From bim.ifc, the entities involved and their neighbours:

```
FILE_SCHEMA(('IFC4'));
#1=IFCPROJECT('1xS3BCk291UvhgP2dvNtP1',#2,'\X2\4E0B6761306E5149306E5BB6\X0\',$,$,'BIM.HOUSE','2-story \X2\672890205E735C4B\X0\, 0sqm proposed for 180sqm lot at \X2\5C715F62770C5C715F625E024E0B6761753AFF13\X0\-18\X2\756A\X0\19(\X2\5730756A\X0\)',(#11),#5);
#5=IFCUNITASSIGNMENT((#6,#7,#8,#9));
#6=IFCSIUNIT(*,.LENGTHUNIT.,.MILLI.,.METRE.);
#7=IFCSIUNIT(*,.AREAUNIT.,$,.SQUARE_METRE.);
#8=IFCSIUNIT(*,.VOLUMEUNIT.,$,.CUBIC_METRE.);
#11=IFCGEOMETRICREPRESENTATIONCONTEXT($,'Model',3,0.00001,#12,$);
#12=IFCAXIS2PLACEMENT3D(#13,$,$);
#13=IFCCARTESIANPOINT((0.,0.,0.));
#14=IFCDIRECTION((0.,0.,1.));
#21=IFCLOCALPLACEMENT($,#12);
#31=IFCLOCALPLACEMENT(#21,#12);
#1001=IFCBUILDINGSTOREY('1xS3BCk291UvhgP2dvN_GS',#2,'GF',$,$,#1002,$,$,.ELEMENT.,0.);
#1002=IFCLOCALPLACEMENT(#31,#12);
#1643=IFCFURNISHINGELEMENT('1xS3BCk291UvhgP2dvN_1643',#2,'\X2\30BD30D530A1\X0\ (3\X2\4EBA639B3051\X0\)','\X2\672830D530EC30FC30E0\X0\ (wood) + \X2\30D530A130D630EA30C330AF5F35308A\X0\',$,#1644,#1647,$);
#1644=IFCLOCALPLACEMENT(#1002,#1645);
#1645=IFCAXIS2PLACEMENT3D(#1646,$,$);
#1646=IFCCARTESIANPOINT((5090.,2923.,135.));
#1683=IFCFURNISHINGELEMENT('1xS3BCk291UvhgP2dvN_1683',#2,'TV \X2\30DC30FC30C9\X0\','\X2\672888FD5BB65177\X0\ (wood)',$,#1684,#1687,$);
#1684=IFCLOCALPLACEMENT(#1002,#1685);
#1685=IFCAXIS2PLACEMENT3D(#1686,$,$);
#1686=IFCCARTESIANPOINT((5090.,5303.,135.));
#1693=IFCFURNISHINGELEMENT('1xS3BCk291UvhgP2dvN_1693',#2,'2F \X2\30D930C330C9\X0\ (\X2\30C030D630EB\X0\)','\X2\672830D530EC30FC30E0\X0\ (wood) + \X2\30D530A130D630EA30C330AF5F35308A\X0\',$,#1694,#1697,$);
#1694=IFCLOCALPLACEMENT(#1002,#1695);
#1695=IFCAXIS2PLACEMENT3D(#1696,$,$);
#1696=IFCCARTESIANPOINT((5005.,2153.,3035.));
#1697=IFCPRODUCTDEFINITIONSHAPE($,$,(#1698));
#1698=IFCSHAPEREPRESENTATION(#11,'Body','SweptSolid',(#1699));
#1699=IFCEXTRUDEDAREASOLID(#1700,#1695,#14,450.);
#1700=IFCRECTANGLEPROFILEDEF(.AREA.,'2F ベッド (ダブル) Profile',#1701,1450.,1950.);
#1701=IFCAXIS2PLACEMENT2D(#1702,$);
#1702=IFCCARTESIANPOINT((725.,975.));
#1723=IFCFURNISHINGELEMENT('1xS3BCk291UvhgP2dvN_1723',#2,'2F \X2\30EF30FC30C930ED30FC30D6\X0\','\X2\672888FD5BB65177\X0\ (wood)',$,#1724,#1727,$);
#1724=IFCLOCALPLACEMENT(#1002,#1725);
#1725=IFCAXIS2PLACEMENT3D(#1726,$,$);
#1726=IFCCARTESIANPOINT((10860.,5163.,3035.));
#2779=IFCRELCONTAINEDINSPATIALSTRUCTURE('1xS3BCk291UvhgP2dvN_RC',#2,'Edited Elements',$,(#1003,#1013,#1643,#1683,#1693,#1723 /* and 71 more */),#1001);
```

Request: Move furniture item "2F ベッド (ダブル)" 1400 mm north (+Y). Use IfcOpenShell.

```python
import ifcopenshell
import ifcopenshell.api.geometry
import ifcopenshell.util.placement

model = ifcopenshell.open("bim.ifc")

item = model.by_guid("1xS3BCk291UvhgP2dvN_1693")
matrix = ifcopenshell.util.placement.get_local_placement(item.ObjectPlacement)
matrix[1, 3] += 1400.0
ifcopenshell.api.geometry.edit_object_placement(model, product=item, matrix=matrix, is_si=False)

print(ifcopenshell.util.placement.get_local_placement(item.ObjectPlacement).round(3) + 0.0)

model.write("bim_updated.ifc")
```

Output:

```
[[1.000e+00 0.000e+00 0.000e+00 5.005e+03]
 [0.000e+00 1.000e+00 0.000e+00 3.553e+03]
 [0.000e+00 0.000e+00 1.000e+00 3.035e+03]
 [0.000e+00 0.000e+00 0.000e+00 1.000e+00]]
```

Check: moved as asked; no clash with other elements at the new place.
